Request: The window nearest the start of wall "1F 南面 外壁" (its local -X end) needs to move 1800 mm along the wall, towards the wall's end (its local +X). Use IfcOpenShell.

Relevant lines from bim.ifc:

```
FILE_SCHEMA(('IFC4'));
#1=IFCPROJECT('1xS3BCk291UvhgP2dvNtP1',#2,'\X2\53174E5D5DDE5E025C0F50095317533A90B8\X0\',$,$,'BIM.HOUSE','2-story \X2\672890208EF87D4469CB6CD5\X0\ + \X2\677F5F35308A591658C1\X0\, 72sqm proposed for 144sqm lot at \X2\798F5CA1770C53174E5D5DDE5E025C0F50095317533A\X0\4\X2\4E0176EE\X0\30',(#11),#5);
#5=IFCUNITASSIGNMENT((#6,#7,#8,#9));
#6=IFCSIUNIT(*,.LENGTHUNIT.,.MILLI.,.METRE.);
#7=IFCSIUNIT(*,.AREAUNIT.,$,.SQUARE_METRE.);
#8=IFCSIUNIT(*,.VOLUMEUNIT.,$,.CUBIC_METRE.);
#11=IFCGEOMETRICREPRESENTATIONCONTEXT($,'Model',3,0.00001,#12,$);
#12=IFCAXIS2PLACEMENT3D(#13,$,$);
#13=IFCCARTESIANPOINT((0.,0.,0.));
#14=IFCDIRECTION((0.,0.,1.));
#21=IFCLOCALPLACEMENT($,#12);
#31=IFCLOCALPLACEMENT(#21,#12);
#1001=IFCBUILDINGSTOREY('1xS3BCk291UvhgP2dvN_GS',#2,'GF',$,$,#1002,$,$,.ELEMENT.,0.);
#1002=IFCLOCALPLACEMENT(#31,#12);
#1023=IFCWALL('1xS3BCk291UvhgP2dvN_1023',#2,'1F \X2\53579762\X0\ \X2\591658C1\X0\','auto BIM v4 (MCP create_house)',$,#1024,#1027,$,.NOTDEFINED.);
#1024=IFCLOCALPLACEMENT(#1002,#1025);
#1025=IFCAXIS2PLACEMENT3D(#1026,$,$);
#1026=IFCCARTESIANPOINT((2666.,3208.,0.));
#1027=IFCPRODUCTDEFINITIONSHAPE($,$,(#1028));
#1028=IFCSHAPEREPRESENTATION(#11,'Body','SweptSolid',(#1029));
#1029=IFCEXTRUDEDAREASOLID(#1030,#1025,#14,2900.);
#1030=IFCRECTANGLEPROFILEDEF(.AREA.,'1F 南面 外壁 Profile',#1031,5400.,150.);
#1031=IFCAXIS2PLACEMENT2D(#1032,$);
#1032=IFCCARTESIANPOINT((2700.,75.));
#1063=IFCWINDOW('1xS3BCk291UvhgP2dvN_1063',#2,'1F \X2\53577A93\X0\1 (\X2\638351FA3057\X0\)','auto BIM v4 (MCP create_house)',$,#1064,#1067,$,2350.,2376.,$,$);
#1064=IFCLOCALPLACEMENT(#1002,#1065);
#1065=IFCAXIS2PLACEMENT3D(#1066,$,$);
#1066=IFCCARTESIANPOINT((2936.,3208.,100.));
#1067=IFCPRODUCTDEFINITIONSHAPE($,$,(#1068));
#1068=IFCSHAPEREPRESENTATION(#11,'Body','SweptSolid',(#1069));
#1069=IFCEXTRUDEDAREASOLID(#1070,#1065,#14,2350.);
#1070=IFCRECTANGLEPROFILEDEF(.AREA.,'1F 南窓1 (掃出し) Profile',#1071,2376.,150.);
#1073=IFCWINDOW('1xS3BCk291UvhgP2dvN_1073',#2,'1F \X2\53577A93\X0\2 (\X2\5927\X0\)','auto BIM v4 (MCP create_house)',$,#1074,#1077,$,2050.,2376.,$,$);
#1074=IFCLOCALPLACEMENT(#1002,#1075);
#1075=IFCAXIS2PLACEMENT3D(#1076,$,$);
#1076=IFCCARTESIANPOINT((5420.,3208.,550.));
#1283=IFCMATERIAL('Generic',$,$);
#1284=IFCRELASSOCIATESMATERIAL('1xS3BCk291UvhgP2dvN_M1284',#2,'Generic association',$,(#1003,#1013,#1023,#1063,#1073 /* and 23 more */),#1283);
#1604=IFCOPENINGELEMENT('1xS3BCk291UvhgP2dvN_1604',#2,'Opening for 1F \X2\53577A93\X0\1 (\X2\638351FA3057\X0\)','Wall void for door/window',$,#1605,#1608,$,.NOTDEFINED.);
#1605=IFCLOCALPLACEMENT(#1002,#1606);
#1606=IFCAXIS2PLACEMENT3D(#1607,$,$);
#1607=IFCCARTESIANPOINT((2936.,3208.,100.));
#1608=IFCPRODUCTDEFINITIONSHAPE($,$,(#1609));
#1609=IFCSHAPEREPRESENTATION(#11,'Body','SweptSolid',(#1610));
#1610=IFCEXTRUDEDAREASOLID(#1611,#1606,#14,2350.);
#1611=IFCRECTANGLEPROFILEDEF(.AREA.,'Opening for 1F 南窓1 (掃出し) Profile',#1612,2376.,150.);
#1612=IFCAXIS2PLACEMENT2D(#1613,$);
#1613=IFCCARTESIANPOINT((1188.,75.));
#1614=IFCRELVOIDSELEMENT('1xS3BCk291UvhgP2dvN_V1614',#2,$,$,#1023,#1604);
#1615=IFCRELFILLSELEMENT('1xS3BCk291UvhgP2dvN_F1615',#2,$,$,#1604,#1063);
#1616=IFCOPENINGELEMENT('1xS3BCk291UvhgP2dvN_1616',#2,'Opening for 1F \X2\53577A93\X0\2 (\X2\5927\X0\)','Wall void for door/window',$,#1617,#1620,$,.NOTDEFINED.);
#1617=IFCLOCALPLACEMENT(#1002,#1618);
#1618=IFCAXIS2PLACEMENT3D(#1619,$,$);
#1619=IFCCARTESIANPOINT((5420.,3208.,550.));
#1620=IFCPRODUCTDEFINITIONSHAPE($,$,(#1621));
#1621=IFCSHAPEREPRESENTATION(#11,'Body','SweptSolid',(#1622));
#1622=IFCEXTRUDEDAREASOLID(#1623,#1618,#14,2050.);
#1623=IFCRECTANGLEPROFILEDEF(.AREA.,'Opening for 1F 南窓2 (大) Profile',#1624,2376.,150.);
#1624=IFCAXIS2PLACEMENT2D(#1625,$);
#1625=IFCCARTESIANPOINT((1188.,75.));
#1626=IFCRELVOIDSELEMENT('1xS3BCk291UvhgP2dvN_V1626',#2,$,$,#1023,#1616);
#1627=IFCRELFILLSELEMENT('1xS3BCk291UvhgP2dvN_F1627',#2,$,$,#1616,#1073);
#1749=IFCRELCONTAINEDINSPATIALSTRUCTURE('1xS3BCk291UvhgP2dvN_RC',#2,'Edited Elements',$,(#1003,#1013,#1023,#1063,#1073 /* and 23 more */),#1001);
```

```python
import ifcopenshell
import ifcopenshell.api.geometry
import ifcopenshell.util.placement
import ifcopenshell.util.unit

model = ifcopenshell.open("bim.ifc")
unit_scale = ifcopenshell.util.unit.calculate_unit_scale(model)

window = model.by_guid("1xS3BCk291UvhgP2dvN_1063")
opening = window.FillsVoids[0].RelatingOpeningElement
wall = opening.VoidsElements[0].RelatingBuildingElement

wall_matrix = ifcopenshell.util.placement.get_local_placement(wall.ObjectPlacement)
shift = wall_matrix[:3, 0] * 1.8 / unit_scale
before = ifcopenshell.util.placement.get_local_placement(window.ObjectPlacement)[:3, 3].copy()

# The window is not placed relative to its opening, so move both.
for product in (opening, window):
    matrix = ifcopenshell.util.placement.get_local_placement(product.ObjectPlacement)
    matrix[:3, 3] += shift
    ifcopenshell.api.geometry.edit_object_placement(model, product=product, matrix=matrix, is_si=False)

after = ifcopenshell.util.placement.get_local_placement(window.ObjectPlacement)[:3, 3]
print("window moved by", (after - before).round(3) + 0.0)

model.write("bim-out.ifc")
```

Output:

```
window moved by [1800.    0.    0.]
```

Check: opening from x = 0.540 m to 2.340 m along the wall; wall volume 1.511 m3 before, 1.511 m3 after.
